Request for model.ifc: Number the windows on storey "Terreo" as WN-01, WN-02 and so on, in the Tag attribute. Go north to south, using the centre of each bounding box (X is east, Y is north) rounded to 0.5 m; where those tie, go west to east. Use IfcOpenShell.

First a look at what the model holds.

```python
import ifcopenshell
import ifcopenshell.util.element
import ifcopenshell.util.placement

model = ifcopenshell.open("model.ifc")
print(model.schema)
storey = next(s for s in model.by_type("IfcBuildingStorey") if s.Name == "Terreo")
windows = [e for e in ifcopenshell.util.element.get_decomposition(storey) if e.is_a("IfcWindow")]
for e in sorted(windows, key=lambda e: e.id()):
    origin = ifcopenshell.util.placement.get_local_placement(e.ObjectPlacement)[:3, 3]
    print(e.id(), e.Tag, e.Name, origin.round(2) + 0.0, sep=" | ")
```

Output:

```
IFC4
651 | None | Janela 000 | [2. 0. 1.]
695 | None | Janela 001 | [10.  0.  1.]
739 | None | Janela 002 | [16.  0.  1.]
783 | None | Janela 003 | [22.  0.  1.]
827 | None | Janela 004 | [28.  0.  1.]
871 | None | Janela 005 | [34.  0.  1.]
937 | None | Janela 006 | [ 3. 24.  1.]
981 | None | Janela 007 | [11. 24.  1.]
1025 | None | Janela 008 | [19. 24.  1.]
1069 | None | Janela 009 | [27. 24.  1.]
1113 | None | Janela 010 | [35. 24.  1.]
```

```python
import ifcopenshell
import ifcopenshell.geom
import ifcopenshell.util.element
import ifcopenshell.util.shape

model = ifcopenshell.open("model.ifc")
settings = ifcopenshell.geom.settings()
settings.set("use-world-coords", True)


def centre(element):
    shape = ifcopenshell.geom.create_shape(settings, element)
    return ifcopenshell.util.shape.get_bbox_centroid(shape.geometry)


storey = next(s for s in model.by_type("IfcBuildingStorey") if s.Name == "Terreo")
windows = [e for e in ifcopenshell.util.element.get_decomposition(storey) if e.is_a("IfcWindow")]

# Insertion points can sit at a corner or the storey origin, so sort by the geometry (in metres).
centres = {e: centre(e) for e in windows}
windows.sort(key=lambda e: (-round(centres[e][1] / 0.5), centres[e][0]))

for i, e in enumerate(windows, start=1):
    number = f"WN-{i:02d}"
    e.Tag = number
    print(e.id(), number)

model.write("model_edited.ifc")
```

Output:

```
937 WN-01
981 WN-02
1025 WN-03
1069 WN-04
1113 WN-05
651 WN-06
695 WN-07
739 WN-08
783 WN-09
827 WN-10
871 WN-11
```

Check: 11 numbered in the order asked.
